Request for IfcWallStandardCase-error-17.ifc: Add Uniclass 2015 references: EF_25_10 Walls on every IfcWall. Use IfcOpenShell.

First a look at what the model holds.

```python
import ifcopenshell

model = ifcopenshell.open("IfcWallStandardCase-error-17.ifc")
print(model.schema)
print("classifications:", [c.Name for c in model.by_type("IfcClassification")])
for ifc_class in ("IfcDoor", "IfcRoof", "IfcStair", "IfcWall", "IfcWindow"):
    print(ifc_class, len(model.by_type(ifc_class)))
```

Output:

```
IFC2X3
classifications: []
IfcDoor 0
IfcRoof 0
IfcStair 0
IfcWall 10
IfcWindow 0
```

```python
import ifcopenshell
import ifcopenshell.api.classification

model = ifcopenshell.open("IfcWallStandardCase-error-17.ifc")

# IFC2X3 requires Source and Edition and has no link from the project to the system.
system = model.create_entity("IfcClassification", Source="NBS", Edition="2015", Name="Uniclass 2015")

codes = {
    "IfcWall": ("EF_25_10", "Walls"),
}
for ifc_class, (code, name) in codes.items():
    products = model.by_type(ifc_class)
    ifcopenshell.api.classification.add_reference(
        model, products=products, classification=system, identification=code, name=name
    )
    print(code, len(products))

model.write("IfcWallStandardCase-error-17_rev.ifc")
```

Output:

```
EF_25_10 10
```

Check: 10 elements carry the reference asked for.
